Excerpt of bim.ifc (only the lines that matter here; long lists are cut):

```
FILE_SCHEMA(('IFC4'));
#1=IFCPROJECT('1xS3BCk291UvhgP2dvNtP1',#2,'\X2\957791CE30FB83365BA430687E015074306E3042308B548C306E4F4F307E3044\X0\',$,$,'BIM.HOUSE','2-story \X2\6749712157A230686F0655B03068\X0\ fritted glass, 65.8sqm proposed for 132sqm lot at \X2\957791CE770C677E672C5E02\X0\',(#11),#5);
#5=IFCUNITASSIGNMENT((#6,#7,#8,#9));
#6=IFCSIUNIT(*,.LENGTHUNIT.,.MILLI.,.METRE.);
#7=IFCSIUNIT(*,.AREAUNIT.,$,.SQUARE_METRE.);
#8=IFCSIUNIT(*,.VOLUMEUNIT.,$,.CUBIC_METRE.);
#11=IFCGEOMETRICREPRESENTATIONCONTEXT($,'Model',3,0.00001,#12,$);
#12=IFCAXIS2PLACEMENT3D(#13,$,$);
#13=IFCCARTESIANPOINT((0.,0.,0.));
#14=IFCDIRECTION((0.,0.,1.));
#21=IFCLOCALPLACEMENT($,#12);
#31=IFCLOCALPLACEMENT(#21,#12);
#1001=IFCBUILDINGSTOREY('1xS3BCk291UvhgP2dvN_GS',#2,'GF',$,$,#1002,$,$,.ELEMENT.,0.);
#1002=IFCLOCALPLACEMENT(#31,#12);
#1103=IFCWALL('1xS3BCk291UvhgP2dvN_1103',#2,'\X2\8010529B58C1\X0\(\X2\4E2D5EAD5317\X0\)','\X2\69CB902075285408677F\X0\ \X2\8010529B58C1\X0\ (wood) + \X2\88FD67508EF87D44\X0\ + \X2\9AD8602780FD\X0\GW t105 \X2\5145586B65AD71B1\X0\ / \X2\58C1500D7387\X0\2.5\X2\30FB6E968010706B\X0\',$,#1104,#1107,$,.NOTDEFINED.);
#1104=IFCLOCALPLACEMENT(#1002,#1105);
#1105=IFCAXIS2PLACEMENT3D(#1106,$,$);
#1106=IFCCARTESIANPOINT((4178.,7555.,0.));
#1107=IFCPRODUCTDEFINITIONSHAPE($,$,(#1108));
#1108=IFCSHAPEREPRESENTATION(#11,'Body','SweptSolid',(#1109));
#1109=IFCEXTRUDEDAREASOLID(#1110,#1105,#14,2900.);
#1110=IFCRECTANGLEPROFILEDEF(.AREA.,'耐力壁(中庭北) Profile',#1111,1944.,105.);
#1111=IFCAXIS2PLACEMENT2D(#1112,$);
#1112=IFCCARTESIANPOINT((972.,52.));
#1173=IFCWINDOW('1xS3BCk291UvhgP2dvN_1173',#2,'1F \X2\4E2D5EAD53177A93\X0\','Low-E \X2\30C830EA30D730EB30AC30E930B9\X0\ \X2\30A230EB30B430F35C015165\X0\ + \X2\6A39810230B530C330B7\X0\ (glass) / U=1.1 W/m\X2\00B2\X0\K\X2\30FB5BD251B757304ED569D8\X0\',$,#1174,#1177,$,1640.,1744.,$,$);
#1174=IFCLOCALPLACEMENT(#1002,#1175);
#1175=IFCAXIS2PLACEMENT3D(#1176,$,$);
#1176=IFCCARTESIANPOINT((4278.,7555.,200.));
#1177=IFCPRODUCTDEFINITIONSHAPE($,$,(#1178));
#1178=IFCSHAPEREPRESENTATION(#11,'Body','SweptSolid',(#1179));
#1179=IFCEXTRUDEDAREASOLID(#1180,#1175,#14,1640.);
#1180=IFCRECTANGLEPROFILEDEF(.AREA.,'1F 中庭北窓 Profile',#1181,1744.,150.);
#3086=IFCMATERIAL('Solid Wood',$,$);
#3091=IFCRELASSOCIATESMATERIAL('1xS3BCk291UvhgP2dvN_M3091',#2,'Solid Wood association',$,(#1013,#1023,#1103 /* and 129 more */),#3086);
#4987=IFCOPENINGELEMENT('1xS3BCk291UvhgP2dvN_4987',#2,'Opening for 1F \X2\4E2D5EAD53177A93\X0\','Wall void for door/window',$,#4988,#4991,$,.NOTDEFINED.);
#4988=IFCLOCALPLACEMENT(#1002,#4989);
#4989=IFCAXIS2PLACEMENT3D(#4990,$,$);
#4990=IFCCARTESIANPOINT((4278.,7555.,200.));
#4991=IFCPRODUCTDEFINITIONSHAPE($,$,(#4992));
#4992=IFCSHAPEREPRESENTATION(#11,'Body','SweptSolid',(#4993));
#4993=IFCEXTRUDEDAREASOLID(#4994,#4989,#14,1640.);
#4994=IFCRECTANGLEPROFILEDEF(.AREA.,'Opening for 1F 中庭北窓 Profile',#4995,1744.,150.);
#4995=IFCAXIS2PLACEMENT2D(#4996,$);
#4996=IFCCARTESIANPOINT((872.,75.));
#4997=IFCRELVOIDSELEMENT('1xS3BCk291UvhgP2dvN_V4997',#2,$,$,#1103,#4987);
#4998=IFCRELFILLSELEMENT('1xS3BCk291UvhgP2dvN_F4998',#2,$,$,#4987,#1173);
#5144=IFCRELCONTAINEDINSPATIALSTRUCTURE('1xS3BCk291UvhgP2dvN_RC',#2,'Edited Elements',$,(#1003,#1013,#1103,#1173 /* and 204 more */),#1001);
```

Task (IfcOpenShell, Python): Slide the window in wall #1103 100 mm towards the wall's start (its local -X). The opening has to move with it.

```python
import ifcopenshell
import ifcopenshell.api.geometry
import ifcopenshell.util.placement
import ifcopenshell.util.unit

model = ifcopenshell.open("bim.ifc")
unit_scale = ifcopenshell.util.unit.calculate_unit_scale(model)

window = model.by_id(1173)
opening = window.FillsVoids[0].RelatingOpeningElement
wall = opening.VoidsElements[0].RelatingBuildingElement

wall_matrix = ifcopenshell.util.placement.get_local_placement(wall.ObjectPlacement)
shift = wall_matrix[:3, 0] * -0.1 / unit_scale
before = ifcopenshell.util.placement.get_local_placement(window.ObjectPlacement)[:3, 3].copy()

# The window is not placed relative to its opening, so move both.
for product in (opening, window):
    matrix = ifcopenshell.util.placement.get_local_placement(product.ObjectPlacement)
    matrix[:3, 3] += shift
    ifcopenshell.api.geometry.edit_object_placement(model, product=product, matrix=matrix, is_si=False)

after = ifcopenshell.util.placement.get_local_placement(window.ObjectPlacement)[:3, 3]
print("window moved by", (after - before).round(3) + 0.0)

model.write("bim-out.ifc")
```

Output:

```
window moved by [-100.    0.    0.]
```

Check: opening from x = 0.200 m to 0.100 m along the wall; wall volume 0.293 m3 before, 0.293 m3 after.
